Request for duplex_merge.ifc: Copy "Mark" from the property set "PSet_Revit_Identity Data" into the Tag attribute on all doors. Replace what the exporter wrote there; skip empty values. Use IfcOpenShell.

First a look at what the model holds.

```python
import ifcopenshell
import ifcopenshell.util.element

model = ifcopenshell.open("duplex_merge.ifc")
print(model.schema)
doors = model.by_type("IfcDoor")
print(len(doors), "doors")
for e in doors[:8]:
    source = ifcopenshell.util.element.get_pset(e, "PSet_Revit_Identity Data", "Mark")
    target = e.Tag
    print(e.id(), repr(source), repr(target), sep=" | ")
```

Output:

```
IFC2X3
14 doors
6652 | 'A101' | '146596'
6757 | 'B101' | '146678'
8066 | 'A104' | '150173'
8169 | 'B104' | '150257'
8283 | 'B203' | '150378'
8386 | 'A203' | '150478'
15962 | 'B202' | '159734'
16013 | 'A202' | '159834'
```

```python
import ifcopenshell
import ifcopenshell.util.element

model = ifcopenshell.open("duplex_merge.ifc")

count = 0
for e in model.by_type("IfcDoor"):
    value = ifcopenshell.util.element.get_pset(e, "PSet_Revit_Identity Data", "Mark")
    current = e.Tag
    if not value or not value.strip() or current == value:
        continue
    e.Tag = value
    count += 1

print(count, "doors updated")

model.write("duplex_merge_updated.ifc")
```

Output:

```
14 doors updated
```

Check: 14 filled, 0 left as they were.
